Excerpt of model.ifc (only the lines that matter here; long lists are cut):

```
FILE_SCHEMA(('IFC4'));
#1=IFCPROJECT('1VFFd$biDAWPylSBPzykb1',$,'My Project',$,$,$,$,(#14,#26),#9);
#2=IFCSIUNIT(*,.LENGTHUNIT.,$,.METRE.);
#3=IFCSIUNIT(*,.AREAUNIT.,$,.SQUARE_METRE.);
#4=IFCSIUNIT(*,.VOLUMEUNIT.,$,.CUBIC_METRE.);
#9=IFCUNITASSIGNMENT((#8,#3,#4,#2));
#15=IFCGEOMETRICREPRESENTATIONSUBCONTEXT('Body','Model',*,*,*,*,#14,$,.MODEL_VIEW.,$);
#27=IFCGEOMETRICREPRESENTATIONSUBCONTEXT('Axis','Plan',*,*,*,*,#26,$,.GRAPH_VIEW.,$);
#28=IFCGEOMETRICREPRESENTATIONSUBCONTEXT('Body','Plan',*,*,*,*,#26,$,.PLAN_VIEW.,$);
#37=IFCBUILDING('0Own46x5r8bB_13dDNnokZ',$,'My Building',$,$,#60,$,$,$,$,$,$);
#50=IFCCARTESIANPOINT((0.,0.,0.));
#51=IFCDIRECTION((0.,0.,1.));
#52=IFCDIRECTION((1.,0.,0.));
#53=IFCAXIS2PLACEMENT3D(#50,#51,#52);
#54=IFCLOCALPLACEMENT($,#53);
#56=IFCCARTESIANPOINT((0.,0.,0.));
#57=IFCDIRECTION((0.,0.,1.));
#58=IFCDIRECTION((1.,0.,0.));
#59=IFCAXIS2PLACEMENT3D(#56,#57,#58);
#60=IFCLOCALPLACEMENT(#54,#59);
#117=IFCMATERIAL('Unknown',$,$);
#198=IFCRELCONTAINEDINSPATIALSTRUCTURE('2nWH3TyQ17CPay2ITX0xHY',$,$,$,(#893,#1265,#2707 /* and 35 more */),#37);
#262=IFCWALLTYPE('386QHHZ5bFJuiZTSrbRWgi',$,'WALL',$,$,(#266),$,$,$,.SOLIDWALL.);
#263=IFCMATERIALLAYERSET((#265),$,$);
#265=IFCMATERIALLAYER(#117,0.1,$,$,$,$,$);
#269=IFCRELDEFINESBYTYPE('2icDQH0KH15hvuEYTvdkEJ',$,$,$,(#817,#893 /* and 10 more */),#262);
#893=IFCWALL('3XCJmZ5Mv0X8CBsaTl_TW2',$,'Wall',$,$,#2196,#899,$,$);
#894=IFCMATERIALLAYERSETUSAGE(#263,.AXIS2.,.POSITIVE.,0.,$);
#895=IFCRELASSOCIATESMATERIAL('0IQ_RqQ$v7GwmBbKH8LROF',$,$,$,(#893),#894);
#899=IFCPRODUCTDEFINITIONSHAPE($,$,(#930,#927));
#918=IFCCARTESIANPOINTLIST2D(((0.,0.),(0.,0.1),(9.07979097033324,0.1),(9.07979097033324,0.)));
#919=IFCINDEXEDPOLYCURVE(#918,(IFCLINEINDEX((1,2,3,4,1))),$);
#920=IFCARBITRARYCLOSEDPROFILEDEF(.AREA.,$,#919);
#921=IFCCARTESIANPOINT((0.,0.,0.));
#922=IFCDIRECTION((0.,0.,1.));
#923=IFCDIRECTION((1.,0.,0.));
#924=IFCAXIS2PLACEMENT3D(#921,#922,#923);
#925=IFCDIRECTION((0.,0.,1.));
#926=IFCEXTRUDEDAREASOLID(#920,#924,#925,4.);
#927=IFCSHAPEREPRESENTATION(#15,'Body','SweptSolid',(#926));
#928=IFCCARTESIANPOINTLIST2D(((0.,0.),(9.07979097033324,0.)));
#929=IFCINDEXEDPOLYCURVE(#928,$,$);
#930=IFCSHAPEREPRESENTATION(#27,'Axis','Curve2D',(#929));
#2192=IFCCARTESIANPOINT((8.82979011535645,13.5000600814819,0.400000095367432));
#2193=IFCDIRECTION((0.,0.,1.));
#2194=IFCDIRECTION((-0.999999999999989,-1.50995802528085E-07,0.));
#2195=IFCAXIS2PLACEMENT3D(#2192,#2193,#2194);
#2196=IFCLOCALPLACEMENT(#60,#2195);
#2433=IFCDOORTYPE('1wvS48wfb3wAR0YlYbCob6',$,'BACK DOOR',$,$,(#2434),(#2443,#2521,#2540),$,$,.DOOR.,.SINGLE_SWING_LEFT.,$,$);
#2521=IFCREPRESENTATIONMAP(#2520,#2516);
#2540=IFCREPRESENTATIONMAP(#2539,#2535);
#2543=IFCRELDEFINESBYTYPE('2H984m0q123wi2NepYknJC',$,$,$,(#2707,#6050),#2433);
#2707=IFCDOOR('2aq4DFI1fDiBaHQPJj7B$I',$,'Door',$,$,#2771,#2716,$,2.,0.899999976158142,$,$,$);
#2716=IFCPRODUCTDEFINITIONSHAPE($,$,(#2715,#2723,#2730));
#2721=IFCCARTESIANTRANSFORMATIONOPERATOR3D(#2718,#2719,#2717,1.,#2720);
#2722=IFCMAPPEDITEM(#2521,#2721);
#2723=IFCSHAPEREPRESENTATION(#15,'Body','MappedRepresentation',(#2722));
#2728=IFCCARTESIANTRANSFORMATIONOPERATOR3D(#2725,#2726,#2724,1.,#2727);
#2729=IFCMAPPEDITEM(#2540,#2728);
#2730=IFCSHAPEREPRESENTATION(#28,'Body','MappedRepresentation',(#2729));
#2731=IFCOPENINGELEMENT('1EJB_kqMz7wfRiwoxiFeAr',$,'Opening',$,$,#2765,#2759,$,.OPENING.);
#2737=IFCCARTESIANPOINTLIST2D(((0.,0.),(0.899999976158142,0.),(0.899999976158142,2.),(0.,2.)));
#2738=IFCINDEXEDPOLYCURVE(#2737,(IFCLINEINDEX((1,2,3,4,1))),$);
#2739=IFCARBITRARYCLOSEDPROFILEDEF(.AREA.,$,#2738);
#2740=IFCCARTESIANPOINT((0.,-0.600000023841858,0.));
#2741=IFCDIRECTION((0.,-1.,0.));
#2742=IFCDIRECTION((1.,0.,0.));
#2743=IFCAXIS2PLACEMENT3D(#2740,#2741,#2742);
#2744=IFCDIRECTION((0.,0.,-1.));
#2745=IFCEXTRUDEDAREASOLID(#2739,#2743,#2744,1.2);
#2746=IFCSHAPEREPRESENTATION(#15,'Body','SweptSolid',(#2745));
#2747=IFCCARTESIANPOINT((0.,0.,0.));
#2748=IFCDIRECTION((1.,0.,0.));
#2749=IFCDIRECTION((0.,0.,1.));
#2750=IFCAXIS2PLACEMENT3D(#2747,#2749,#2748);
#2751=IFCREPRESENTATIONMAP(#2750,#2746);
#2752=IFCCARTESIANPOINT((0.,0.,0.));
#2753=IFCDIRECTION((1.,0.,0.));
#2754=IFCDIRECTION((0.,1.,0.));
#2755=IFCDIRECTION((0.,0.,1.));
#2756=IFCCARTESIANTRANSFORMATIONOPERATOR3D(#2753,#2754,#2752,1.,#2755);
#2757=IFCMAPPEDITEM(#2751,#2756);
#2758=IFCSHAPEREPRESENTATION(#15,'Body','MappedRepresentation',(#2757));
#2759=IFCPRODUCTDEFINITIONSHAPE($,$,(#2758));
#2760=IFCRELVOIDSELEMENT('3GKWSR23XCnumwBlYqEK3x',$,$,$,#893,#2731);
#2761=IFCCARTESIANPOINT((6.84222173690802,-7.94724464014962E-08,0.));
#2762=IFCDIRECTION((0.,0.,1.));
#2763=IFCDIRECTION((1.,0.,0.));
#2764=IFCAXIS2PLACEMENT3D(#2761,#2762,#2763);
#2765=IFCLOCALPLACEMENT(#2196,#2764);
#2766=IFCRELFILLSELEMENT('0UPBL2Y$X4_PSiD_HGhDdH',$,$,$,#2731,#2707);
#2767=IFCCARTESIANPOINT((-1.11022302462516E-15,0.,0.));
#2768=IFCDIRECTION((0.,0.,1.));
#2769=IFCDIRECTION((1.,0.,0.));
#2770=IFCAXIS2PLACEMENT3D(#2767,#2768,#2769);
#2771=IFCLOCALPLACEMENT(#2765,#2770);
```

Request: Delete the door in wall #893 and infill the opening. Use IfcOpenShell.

```python
import ifcopenshell
import ifcopenshell.api.feature
import ifcopenshell.api.root
import ifcopenshell.geom
import ifcopenshell.util.shape

model = ifcopenshell.open("model.ifc")
settings = ifcopenshell.geom.settings()


def volume(element):
    """Net volume in cubic metres, openings subtracted."""
    shape = ifcopenshell.geom.create_shape(settings, element)
    return ifcopenshell.util.shape.get_volume(shape.geometry)


door = model.by_id(2707)
opening = door.FillsVoids[0].RelatingOpeningElement
wall = opening.VoidsElements[0].RelatingBuildingElement
before = volume(wall)

ifcopenshell.api.root.remove_product(model, product=door)
ifcopenshell.api.feature.remove_feature(model, feature=opening)

after = volume(wall)

print(f"wall volume {before:.3f} -> {after:.3f} m3")

model.write("model_edited.ifc")
```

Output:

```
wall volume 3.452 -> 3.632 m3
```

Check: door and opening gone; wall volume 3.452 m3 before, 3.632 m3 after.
